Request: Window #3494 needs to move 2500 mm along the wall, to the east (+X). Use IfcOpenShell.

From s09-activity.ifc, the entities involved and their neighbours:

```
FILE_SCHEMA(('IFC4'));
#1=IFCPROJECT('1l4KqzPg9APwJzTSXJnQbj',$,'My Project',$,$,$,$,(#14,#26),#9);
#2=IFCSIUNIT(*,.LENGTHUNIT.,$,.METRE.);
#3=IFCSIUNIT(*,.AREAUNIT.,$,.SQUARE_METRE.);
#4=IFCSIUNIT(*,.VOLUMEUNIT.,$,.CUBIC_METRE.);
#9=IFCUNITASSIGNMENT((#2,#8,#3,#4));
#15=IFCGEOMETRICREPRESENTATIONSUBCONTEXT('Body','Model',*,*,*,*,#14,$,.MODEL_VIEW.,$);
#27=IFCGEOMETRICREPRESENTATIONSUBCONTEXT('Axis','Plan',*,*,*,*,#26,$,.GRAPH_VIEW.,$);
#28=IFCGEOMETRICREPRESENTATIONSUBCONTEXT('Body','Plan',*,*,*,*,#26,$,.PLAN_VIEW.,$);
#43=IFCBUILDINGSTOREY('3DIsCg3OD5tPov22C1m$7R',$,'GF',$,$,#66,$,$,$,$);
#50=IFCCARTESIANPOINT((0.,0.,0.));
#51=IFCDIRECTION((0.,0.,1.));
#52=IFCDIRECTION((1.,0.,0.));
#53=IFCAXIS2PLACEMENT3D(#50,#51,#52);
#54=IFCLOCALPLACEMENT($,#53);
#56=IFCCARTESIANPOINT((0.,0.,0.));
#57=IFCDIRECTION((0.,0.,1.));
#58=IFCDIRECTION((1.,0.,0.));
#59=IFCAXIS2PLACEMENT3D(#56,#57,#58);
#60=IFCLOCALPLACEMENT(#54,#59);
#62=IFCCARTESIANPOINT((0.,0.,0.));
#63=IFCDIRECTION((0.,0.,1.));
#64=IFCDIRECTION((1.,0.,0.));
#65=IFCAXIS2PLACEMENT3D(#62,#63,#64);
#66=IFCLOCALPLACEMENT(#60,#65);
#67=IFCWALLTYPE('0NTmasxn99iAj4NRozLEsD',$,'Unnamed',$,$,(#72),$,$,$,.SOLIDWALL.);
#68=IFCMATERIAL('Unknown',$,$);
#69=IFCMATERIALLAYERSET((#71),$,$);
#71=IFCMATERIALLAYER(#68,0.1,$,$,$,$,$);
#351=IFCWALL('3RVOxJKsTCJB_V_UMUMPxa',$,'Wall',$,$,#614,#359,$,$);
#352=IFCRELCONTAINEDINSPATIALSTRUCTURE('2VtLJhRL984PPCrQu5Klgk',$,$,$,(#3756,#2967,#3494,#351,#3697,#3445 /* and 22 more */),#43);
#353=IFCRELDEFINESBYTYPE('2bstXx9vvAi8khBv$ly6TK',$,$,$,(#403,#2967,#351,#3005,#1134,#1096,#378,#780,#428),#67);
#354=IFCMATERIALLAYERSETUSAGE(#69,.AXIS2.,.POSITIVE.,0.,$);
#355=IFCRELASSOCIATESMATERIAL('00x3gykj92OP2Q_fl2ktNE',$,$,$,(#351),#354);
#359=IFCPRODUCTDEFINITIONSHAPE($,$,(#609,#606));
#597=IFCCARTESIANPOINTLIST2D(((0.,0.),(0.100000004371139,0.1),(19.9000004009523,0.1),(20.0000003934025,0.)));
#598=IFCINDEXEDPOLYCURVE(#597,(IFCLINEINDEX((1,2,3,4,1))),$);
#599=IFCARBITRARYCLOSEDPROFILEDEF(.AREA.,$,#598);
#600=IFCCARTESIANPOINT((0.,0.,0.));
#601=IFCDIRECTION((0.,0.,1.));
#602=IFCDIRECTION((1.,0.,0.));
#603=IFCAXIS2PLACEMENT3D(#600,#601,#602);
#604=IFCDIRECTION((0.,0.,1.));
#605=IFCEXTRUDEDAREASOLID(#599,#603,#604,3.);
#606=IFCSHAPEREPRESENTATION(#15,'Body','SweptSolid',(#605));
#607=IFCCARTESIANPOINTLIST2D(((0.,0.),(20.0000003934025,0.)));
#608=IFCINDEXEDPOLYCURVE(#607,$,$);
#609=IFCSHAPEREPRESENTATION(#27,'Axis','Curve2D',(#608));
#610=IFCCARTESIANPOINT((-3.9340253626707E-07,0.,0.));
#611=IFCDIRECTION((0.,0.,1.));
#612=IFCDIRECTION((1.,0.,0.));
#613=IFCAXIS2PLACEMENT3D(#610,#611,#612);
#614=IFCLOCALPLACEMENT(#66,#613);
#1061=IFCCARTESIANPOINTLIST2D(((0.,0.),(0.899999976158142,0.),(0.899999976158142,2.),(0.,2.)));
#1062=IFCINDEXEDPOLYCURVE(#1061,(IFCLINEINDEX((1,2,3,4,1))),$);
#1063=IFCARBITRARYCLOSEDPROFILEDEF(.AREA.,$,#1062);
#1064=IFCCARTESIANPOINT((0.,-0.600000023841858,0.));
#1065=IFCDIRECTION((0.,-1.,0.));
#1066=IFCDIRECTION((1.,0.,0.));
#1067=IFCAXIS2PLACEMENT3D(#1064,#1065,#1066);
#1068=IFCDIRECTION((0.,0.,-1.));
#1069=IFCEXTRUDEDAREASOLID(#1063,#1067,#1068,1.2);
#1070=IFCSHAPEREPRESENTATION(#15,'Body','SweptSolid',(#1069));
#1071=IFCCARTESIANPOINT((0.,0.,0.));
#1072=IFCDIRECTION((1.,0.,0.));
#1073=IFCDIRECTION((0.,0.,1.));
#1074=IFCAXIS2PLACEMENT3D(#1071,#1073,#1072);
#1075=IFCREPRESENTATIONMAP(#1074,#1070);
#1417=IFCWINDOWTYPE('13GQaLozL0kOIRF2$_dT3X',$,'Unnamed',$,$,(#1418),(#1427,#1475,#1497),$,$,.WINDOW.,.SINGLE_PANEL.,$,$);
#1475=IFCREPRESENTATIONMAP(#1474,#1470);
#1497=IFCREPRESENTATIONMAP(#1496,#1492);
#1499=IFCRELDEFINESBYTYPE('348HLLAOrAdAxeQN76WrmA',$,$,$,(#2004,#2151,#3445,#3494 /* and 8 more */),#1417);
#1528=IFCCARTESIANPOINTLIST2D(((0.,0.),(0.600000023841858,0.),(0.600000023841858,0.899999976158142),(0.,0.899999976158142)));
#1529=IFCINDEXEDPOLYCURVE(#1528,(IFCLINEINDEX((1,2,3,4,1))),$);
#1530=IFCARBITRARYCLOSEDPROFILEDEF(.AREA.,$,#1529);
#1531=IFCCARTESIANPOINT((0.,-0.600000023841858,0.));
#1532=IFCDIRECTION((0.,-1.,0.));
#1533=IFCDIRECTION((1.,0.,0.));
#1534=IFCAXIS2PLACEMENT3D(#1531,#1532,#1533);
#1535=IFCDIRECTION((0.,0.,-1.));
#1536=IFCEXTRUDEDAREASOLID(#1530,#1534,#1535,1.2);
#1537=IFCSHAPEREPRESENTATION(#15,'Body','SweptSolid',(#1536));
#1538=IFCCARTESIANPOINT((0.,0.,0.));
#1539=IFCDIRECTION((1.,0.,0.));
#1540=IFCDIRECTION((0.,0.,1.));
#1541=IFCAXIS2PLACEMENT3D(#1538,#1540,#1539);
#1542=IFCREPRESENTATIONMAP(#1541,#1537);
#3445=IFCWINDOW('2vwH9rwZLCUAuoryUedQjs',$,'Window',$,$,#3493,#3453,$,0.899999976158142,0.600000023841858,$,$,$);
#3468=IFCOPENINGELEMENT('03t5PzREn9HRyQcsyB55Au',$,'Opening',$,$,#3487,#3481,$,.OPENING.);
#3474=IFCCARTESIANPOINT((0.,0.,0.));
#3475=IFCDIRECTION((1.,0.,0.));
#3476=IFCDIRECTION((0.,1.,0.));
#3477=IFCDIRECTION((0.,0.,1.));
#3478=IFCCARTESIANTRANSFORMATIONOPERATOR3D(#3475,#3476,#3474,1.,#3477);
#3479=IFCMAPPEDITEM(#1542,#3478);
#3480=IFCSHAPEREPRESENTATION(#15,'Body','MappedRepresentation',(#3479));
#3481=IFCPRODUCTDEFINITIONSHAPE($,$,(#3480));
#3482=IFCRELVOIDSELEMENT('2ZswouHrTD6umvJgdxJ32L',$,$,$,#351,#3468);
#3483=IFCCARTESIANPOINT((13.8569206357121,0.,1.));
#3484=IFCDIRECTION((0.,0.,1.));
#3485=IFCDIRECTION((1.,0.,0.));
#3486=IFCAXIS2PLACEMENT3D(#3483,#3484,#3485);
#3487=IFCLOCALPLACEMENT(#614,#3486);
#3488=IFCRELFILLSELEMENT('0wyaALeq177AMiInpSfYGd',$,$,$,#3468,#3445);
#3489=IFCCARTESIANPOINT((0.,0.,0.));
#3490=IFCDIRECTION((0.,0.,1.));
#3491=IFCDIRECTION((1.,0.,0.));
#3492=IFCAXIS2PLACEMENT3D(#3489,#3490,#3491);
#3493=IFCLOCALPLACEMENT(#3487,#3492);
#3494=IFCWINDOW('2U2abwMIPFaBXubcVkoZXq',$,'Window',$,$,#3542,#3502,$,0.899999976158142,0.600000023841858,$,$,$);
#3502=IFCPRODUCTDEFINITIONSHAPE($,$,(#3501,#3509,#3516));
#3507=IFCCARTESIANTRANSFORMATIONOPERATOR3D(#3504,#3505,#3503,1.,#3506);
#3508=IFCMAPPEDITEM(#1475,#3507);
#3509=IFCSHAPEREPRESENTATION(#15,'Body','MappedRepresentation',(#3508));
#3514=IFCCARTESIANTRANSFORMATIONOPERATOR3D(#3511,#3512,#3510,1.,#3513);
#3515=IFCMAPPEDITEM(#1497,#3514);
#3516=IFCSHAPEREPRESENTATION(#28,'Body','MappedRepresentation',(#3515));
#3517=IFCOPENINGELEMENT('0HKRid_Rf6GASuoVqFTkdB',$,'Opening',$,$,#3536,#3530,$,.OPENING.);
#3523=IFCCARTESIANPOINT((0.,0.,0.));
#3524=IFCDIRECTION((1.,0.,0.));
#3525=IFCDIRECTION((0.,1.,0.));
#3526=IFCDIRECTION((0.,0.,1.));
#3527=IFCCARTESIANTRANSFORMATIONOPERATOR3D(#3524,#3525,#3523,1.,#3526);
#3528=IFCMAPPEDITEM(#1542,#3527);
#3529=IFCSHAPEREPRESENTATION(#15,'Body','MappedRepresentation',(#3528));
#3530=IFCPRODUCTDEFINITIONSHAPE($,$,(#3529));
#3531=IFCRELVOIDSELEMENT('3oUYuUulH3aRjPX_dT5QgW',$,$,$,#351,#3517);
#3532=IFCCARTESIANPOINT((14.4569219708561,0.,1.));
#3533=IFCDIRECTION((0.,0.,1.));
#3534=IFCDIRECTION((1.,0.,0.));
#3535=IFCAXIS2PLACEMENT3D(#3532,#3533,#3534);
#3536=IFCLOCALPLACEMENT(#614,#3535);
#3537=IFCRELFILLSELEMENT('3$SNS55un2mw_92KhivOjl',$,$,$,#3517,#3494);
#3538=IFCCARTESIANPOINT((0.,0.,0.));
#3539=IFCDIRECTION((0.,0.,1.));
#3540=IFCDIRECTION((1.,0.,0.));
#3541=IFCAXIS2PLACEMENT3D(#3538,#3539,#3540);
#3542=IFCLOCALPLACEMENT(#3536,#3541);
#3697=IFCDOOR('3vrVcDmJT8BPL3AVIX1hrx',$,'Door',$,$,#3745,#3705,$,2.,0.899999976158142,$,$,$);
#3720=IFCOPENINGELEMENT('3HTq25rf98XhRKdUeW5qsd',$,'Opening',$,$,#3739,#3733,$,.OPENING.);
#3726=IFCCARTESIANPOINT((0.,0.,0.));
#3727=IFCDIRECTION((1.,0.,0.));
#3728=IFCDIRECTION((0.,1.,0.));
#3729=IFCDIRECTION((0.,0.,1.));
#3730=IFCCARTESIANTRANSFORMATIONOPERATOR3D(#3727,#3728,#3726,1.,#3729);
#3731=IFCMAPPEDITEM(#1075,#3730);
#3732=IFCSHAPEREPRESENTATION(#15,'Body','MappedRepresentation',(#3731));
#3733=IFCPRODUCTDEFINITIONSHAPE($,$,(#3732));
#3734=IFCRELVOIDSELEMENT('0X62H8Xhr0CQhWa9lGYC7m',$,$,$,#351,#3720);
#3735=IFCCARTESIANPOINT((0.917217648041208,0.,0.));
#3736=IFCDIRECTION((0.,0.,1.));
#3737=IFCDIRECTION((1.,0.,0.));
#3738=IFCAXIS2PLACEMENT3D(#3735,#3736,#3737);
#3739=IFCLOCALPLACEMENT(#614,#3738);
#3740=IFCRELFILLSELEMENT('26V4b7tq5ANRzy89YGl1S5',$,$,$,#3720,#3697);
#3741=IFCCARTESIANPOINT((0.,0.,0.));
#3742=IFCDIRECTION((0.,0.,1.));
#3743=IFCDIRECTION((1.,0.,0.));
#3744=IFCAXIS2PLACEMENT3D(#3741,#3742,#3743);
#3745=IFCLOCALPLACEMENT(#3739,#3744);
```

```python
import ifcopenshell
import ifcopenshell.api.geometry
import ifcopenshell.util.placement
import ifcopenshell.util.unit

model = ifcopenshell.open("s09-activity.ifc")
unit_scale = ifcopenshell.util.unit.calculate_unit_scale(model)

window = model.by_guid("2U2abwMIPFaBXubcVkoZXq")
opening = window.FillsVoids[0].RelatingOpeningElement
wall = opening.VoidsElements[0].RelatingBuildingElement

wall_matrix = ifcopenshell.util.placement.get_local_placement(wall.ObjectPlacement)
shift = wall_matrix[:3, 0] * 2.5 / unit_scale
before = ifcopenshell.util.placement.get_local_placement(window.ObjectPlacement)[:3, 3].copy()

# The window is placed relative to its opening, so it follows when the opening moves.
matrix = ifcopenshell.util.placement.get_local_placement(opening.ObjectPlacement)
matrix[:3, 3] += shift
ifcopenshell.api.geometry.edit_object_placement(
    model, product=opening, matrix=matrix, is_si=False, should_transform_children=True
)

after = ifcopenshell.util.placement.get_local_placement(window.ObjectPlacement)[:3, 3]
print("window moved by", (after - before).round(3) + 0.0)

model.write("s09-activity_updated.ifc")
```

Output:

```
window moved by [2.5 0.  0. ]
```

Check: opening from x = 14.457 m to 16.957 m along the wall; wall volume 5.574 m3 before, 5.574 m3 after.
